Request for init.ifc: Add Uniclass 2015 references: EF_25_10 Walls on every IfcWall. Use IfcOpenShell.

First a look at what the model holds.

```python
import ifcopenshell

model = ifcopenshell.open("init.ifc")
print(model.schema)
print("classifications:", [c.Name for c in model.by_type("IfcClassification")])
for ifc_class in ("IfcDoor", "IfcRoof", "IfcStair", "IfcWall", "IfcWindow"):
    print(ifc_class, len(model.by_type(ifc_class)))
```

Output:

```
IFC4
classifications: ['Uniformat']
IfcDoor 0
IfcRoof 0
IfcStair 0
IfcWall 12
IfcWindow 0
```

```python
import ifcopenshell
import ifcopenshell.api.classification

model = ifcopenshell.open("init.ifc")

system = ifcopenshell.api.classification.add_classification(model, classification="Uniclass 2015")

codes = {
    "IfcWall": ("EF_25_10", "Walls"),
}
for ifc_class, (code, name) in codes.items():
    products = model.by_type(ifc_class)
    ifcopenshell.api.classification.add_reference(
        model, products=products, classification=system, identification=code, name=name
    )
    print(code, len(products))

model.write("init_v2.ifc")
```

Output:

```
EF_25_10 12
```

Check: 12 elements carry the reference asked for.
